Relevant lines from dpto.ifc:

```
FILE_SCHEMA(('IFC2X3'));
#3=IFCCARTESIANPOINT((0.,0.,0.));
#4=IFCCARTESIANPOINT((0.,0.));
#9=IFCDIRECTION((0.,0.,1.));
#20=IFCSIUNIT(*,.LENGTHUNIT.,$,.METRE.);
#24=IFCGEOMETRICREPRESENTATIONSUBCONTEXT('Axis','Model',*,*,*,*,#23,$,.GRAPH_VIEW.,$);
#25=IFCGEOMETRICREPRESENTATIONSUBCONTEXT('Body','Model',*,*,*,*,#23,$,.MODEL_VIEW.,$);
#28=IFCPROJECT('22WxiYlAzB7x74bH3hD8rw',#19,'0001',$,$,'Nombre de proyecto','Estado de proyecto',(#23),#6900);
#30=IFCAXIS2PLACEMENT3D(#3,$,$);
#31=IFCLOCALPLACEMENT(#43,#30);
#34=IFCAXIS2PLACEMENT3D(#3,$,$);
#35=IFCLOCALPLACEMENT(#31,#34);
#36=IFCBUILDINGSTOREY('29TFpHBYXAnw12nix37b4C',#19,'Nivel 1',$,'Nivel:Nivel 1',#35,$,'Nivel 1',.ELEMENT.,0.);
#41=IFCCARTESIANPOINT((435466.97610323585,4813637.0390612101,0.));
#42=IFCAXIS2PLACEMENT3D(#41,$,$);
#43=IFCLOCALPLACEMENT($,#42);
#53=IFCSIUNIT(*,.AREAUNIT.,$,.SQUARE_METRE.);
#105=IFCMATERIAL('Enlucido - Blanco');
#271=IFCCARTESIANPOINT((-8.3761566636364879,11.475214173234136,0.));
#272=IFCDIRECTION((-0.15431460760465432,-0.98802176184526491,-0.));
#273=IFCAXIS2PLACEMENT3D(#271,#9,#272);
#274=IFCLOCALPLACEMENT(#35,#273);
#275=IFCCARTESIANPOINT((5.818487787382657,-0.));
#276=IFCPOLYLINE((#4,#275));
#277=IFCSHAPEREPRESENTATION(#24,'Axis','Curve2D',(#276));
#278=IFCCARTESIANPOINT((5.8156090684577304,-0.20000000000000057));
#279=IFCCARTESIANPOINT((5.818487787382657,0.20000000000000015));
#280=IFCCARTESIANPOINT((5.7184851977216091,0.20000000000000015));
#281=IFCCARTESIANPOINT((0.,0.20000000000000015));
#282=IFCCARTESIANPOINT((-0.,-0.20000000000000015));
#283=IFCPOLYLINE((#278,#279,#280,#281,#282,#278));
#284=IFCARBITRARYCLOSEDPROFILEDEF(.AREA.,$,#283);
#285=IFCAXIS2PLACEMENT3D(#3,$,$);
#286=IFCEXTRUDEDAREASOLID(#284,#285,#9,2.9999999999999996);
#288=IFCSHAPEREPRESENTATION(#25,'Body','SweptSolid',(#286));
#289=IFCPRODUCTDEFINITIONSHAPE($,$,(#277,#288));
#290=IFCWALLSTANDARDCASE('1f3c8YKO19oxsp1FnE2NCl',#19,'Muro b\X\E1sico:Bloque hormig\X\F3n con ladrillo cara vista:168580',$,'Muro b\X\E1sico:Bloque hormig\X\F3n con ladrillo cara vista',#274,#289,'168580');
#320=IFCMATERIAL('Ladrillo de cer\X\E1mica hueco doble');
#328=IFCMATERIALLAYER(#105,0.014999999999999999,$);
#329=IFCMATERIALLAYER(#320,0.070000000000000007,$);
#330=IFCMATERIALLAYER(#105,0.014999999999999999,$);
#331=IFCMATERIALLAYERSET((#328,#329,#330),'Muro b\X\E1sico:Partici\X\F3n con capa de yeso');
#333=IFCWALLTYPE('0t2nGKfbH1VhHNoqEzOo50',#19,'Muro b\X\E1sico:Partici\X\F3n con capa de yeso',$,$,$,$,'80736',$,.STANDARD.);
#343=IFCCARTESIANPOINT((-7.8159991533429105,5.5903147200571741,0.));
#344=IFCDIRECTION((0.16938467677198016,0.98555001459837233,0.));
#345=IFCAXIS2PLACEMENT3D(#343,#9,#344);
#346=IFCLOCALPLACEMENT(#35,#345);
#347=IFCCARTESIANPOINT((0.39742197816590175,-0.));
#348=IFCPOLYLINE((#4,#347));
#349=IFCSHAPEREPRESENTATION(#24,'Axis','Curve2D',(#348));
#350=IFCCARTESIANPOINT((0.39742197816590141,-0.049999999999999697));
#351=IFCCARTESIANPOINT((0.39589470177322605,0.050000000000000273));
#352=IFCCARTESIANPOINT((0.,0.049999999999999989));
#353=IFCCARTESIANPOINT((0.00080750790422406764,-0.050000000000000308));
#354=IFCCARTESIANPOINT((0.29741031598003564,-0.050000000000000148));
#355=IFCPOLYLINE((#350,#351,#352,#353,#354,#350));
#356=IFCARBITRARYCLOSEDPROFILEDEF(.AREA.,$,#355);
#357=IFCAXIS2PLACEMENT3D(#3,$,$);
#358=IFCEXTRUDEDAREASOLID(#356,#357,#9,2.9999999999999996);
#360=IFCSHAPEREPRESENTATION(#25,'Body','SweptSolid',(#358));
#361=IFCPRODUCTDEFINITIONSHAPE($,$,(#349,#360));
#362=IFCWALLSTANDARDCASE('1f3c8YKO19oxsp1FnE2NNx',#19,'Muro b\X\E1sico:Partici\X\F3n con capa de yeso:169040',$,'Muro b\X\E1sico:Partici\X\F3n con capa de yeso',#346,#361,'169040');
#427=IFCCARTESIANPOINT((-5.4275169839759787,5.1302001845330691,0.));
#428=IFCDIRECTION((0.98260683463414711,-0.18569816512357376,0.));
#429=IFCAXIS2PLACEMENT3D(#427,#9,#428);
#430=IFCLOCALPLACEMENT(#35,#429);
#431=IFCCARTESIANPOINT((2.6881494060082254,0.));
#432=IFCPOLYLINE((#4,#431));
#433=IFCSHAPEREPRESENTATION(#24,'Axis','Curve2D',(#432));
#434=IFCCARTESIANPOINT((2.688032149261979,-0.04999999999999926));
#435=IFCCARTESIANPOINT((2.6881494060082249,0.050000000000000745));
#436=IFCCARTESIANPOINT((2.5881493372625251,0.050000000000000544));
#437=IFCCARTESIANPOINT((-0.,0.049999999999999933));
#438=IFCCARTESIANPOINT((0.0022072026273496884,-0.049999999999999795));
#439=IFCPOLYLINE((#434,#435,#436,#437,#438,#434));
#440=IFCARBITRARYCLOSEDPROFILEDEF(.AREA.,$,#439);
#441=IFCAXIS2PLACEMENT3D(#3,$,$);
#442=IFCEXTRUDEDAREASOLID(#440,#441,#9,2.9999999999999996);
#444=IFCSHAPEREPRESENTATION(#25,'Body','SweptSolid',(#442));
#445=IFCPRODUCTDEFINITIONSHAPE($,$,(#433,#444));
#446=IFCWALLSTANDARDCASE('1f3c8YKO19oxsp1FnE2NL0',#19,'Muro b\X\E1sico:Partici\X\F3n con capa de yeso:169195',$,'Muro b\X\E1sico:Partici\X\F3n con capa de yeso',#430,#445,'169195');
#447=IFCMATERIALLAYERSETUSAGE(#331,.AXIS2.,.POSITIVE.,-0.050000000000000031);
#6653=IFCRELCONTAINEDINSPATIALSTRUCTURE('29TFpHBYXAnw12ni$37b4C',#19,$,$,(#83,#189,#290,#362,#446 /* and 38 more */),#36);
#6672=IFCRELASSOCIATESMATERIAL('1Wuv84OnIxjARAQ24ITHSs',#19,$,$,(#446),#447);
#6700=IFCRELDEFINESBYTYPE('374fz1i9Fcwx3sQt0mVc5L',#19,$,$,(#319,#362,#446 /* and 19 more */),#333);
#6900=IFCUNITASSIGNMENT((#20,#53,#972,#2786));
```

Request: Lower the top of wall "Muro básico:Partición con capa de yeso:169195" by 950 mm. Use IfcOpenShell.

```python
import ifcopenshell
import ifcopenshell.geom
import ifcopenshell.util.representation
import ifcopenshell.util.shape

model = ifcopenshell.open("dpto.ifc")
settings = ifcopenshell.geom.settings()


def volume(element):
    """Net volume in cubic metres, openings subtracted."""
    shape = ifcopenshell.geom.create_shape(settings, element)
    return ifcopenshell.util.shape.get_volume(shape.geometry)


wall = model.by_guid("1f3c8YKO19oxsp1FnE2NL0")
before = volume(wall)

body = ifcopenshell.util.representation.get_representation(wall, "Model", "Body")
solid = body.Items[0]
old_height = solid.Depth
solid.Depth -= 0.95
after = volume(wall)

print(f"height {old_height:g} -> {solid.Depth:g}, volume {before:.3f} -> {after:.3f} m3")

model.write("dpto_v2.ifc")
```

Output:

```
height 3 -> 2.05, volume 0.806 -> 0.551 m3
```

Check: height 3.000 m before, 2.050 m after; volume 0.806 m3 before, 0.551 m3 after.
